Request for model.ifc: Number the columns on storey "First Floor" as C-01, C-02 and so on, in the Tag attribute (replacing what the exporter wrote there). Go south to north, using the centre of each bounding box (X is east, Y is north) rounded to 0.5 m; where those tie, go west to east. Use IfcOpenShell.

First a look at what the model holds.

```python
import ifcopenshell
import ifcopenshell.util.element
import ifcopenshell.util.placement

model = ifcopenshell.open("model.ifc")
print(model.schema)
storey = next(s for s in model.by_type("IfcBuildingStorey") if s.Name == "First Floor")
columns = [e for e in ifcopenshell.util.element.get_decomposition(storey) if e.is_a("IfcColumn")]
for e in sorted(columns, key=lambda e: e.id()):
    origin = ifcopenshell.util.placement.get_local_placement(e.ObjectPlacement)[:3, 3]
    print(e.id(), e.Tag, e.Name, origin.round(2) + 0.0, sep=" | ")
```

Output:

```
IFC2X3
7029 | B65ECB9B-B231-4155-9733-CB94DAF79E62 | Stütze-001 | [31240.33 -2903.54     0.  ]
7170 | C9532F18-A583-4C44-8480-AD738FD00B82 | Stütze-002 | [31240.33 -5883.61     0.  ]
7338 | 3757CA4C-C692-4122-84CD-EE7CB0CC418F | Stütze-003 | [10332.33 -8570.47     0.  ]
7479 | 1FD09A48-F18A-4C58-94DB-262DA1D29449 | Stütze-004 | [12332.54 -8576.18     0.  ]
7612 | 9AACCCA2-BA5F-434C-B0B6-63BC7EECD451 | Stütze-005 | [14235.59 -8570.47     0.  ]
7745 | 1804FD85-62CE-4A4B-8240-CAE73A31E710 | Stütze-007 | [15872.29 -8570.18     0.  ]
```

```python
import ifcopenshell
import ifcopenshell.geom
import ifcopenshell.util.element
import ifcopenshell.util.shape

model = ifcopenshell.open("model.ifc")
settings = ifcopenshell.geom.settings()
settings.set("use-world-coords", True)


def centre(element):
    shape = ifcopenshell.geom.create_shape(settings, element)
    return ifcopenshell.util.shape.get_bbox_centroid(shape.geometry)


storey = next(s for s in model.by_type("IfcBuildingStorey") if s.Name == "First Floor")
columns = [e for e in ifcopenshell.util.element.get_decomposition(storey) if e.is_a("IfcColumn")]

# Insertion points can sit at a corner or the storey origin, so sort by the geometry (in metres).
centres = {e: centre(e) for e in columns}
columns.sort(key=lambda e: (round(centres[e][1] / 0.5), centres[e][0]))

for i, e in enumerate(columns, start=1):
    number = f"C-{i:02d}"
    e.Tag = number
    print(e.id(), number)

model.write("model_updated.ifc")
```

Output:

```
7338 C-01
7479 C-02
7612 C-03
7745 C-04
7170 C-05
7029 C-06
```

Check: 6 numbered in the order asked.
